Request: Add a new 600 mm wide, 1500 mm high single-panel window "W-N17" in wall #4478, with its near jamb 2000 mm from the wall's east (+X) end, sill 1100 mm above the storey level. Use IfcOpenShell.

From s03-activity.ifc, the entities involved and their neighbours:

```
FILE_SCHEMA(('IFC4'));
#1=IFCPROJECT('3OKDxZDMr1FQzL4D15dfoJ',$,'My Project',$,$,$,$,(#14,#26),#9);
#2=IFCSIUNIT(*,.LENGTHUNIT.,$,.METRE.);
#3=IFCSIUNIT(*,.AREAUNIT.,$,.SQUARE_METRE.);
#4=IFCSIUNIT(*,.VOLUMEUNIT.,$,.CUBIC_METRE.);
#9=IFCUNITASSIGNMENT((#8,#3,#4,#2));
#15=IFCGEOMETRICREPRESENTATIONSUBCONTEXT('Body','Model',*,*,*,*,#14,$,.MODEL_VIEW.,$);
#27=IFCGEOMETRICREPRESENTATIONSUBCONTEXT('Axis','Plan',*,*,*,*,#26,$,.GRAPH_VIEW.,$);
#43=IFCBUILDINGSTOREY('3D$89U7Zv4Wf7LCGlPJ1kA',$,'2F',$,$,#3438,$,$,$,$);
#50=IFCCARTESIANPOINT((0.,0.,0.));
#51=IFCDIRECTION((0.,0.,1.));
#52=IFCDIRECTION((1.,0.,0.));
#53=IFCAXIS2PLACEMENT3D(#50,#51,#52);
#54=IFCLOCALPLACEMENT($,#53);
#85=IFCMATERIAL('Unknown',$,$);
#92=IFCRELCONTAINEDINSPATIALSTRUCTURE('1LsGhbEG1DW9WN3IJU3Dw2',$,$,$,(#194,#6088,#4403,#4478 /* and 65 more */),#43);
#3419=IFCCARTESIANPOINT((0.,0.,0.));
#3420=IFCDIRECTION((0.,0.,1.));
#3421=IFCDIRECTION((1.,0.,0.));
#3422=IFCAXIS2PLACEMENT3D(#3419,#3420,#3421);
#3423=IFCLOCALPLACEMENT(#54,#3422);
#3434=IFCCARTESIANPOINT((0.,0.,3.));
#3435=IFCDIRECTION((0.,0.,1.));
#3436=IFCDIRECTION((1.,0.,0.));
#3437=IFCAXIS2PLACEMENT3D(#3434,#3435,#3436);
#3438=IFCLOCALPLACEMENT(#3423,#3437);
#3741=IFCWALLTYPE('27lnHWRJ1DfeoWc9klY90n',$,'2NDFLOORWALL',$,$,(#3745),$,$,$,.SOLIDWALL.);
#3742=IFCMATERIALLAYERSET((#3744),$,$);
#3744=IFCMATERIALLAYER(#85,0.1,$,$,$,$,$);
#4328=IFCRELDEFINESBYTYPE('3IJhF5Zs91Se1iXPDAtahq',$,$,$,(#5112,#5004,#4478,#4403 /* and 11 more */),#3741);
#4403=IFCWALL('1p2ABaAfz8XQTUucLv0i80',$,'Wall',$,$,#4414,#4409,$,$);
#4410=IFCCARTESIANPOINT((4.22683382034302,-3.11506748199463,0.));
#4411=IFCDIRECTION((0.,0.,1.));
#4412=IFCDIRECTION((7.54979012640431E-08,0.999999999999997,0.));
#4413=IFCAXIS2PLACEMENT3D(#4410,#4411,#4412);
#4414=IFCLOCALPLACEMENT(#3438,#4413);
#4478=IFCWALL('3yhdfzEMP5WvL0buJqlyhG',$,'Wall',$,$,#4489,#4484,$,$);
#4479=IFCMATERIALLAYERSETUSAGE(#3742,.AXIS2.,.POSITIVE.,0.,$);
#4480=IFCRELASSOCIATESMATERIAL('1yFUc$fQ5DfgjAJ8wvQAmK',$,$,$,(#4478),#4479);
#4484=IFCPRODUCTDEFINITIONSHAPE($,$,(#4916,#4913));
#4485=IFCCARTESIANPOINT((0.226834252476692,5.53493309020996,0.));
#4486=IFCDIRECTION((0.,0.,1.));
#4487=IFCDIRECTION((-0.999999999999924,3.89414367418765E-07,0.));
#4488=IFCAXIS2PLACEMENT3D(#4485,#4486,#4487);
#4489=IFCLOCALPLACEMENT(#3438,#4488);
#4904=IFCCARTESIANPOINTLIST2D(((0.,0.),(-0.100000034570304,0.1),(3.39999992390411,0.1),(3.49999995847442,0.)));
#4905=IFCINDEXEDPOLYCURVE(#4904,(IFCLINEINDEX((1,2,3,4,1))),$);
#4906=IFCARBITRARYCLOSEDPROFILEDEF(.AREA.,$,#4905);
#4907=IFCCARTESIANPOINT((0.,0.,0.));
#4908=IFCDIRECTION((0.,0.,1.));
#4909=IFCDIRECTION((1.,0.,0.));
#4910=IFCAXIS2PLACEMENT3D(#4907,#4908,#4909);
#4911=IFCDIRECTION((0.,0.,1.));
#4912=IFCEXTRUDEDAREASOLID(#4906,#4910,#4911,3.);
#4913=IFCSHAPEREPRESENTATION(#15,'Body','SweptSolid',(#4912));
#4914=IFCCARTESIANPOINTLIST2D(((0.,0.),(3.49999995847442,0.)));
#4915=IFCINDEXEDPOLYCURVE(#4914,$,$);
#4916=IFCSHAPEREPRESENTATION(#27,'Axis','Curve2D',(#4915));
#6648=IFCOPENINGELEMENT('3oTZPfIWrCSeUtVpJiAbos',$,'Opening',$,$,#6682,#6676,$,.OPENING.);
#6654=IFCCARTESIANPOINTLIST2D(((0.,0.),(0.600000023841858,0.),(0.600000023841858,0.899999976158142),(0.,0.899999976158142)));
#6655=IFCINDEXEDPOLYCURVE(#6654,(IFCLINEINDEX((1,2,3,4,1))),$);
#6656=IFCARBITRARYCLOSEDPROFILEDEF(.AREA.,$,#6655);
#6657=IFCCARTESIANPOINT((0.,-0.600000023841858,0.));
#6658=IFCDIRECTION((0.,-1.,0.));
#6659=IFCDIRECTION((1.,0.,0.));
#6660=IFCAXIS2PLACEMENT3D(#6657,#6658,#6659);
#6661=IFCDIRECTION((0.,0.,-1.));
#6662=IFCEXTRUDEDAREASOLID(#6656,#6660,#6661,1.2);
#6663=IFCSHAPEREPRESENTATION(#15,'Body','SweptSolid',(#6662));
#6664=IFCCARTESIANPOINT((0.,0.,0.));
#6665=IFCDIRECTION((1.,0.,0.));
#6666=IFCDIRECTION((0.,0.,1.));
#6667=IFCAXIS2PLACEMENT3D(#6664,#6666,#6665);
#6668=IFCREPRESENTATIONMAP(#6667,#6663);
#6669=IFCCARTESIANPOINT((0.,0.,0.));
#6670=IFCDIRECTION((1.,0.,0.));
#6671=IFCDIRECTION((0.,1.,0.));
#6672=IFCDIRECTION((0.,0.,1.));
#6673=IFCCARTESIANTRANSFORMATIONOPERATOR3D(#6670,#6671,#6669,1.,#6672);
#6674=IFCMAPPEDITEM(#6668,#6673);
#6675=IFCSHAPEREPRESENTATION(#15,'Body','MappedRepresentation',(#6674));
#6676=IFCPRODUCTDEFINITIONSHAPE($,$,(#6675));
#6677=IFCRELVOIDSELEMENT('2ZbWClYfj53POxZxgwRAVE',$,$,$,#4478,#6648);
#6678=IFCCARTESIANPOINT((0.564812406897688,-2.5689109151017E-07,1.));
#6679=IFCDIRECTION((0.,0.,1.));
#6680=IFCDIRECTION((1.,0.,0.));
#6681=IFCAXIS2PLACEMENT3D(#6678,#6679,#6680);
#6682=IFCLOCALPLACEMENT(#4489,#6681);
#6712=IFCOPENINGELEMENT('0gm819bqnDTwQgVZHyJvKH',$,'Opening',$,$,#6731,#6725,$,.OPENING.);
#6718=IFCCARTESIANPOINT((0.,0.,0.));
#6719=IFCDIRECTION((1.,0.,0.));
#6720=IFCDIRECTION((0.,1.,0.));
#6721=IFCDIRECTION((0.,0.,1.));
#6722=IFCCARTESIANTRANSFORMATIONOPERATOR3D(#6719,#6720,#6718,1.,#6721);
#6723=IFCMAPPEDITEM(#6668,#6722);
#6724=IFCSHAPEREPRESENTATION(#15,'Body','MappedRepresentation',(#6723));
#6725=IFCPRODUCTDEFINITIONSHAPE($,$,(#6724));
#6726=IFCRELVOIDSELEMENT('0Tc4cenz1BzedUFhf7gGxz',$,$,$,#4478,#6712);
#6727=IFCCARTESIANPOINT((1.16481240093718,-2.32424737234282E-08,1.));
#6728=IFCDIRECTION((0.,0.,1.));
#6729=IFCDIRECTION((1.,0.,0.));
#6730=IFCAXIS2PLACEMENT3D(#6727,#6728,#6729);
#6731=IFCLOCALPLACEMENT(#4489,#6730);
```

```python
import numpy as np
import ifcopenshell
import ifcopenshell.api.feature
import ifcopenshell.api.geometry
import ifcopenshell.api.root
import ifcopenshell.api.spatial
import ifcopenshell.geom
import ifcopenshell.util.element
import ifcopenshell.util.placement
import ifcopenshell.util.representation
import ifcopenshell.util.shape
import ifcopenshell.util.unit

model = ifcopenshell.open("s03-activity.ifc")
unit_scale = ifcopenshell.util.unit.calculate_unit_scale(model)
settings = ifcopenshell.geom.settings()


def volume(element):
    """Net volume in cubic metres, openings subtracted."""
    shape = ifcopenshell.geom.create_shape(settings, element)
    return ifcopenshell.util.shape.get_volume(shape.geometry)


wall = model.by_guid("3yhdfzEMP5WvL0buJqlyhG")
storey = ifcopenshell.util.element.get_container(wall, ifc_class="IfcBuildingStorey")
context = ifcopenshell.util.representation.get_context(model, "Model", "Body", "MODEL_VIEW")
before = volume(wall)

width, height, from_end, sill = 0.6, 1.5, 2, 1.1  # metres

# The wall runs along its own X axis, and the end named is its -X end.
wall_shape = ifcopenshell.geom.create_shape(settings, wall)
x, y, z = ifcopenshell.util.shape.get_vertices(wall_shape.geometry).T
start = x.min() + from_end
face, thickness = float(y.min()), float(y.max() - y.min())
wall_matrix = ifcopenshell.util.placement.get_local_placement(wall.ObjectPlacement)
level = ifcopenshell.util.placement.get_local_placement(storey.ObjectPlacement)[2, 3]


def in_wall(x, y):
    """Placement at x, y metres in the wall's axes, at sill height."""
    matrix = wall_matrix.copy()
    matrix[:, 3] = wall_matrix @ np.array([x / unit_scale, y / unit_scale, 0.0, 1.0])
    matrix[2, 3] = level + sill / unit_scale
    return matrix


# Opening: a box that overshoots both wall faces by 50 mm.
opening = ifcopenshell.api.root.create_entity(model, ifc_class="IfcOpeningElement", predefined_type="OPENING")
box = ifcopenshell.api.geometry.add_wall_representation(
    model, context=context, length=width, height=height, thickness=thickness + 0.1
)
ifcopenshell.api.geometry.assign_representation(model, product=opening, representation=box)
ifcopenshell.api.geometry.edit_object_placement(model, product=opening, matrix=in_wall(start, face - 0.05), is_si=False)
ifcopenshell.api.feature.add_feature(model, feature=opening, element=wall)

window = ifcopenshell.api.root.create_entity(model, ifc_class="IfcWindow", name="W-N17", predefined_type="WINDOW")
window.OverallWidth, window.OverallHeight = width / unit_scale, height / unit_scale
window.PartitioningType = "SINGLE_PANEL"
body = ifcopenshell.api.geometry.add_window_representation(
    model,
    context=context,
    overall_width=window.OverallWidth,
    overall_height=window.OverallHeight,
    partition_type="SINGLE_PANEL",
)
ifcopenshell.api.geometry.assign_representation(model, product=window, representation=body)
ifcopenshell.api.spatial.assign_container(model, products=[window], relating_structure=storey)
ifcopenshell.api.feature.add_filling(model, opening=opening, element=window)

# Centre the window in the wall's thickness.
ifcopenshell.api.geometry.edit_object_placement(model, product=window, matrix=in_wall(start, face), is_si=False)
window_shape = ifcopenshell.geom.create_shape(settings, window)
depth = ifcopenshell.util.shape.get_vertices(window_shape.geometry)[:, 1]
offset = face + thickness / 2 - (depth.min() + depth.max()) / 2
ifcopenshell.api.geometry.edit_object_placement(model, product=window, matrix=in_wall(start, offset), is_si=False)

after = volume(wall)

print(f"wall volume {before:.3f} -> {after:.3f} m3")

model.write("s03-activity_edited.ifc")
```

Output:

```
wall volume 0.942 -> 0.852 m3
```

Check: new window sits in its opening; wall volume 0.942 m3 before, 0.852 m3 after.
